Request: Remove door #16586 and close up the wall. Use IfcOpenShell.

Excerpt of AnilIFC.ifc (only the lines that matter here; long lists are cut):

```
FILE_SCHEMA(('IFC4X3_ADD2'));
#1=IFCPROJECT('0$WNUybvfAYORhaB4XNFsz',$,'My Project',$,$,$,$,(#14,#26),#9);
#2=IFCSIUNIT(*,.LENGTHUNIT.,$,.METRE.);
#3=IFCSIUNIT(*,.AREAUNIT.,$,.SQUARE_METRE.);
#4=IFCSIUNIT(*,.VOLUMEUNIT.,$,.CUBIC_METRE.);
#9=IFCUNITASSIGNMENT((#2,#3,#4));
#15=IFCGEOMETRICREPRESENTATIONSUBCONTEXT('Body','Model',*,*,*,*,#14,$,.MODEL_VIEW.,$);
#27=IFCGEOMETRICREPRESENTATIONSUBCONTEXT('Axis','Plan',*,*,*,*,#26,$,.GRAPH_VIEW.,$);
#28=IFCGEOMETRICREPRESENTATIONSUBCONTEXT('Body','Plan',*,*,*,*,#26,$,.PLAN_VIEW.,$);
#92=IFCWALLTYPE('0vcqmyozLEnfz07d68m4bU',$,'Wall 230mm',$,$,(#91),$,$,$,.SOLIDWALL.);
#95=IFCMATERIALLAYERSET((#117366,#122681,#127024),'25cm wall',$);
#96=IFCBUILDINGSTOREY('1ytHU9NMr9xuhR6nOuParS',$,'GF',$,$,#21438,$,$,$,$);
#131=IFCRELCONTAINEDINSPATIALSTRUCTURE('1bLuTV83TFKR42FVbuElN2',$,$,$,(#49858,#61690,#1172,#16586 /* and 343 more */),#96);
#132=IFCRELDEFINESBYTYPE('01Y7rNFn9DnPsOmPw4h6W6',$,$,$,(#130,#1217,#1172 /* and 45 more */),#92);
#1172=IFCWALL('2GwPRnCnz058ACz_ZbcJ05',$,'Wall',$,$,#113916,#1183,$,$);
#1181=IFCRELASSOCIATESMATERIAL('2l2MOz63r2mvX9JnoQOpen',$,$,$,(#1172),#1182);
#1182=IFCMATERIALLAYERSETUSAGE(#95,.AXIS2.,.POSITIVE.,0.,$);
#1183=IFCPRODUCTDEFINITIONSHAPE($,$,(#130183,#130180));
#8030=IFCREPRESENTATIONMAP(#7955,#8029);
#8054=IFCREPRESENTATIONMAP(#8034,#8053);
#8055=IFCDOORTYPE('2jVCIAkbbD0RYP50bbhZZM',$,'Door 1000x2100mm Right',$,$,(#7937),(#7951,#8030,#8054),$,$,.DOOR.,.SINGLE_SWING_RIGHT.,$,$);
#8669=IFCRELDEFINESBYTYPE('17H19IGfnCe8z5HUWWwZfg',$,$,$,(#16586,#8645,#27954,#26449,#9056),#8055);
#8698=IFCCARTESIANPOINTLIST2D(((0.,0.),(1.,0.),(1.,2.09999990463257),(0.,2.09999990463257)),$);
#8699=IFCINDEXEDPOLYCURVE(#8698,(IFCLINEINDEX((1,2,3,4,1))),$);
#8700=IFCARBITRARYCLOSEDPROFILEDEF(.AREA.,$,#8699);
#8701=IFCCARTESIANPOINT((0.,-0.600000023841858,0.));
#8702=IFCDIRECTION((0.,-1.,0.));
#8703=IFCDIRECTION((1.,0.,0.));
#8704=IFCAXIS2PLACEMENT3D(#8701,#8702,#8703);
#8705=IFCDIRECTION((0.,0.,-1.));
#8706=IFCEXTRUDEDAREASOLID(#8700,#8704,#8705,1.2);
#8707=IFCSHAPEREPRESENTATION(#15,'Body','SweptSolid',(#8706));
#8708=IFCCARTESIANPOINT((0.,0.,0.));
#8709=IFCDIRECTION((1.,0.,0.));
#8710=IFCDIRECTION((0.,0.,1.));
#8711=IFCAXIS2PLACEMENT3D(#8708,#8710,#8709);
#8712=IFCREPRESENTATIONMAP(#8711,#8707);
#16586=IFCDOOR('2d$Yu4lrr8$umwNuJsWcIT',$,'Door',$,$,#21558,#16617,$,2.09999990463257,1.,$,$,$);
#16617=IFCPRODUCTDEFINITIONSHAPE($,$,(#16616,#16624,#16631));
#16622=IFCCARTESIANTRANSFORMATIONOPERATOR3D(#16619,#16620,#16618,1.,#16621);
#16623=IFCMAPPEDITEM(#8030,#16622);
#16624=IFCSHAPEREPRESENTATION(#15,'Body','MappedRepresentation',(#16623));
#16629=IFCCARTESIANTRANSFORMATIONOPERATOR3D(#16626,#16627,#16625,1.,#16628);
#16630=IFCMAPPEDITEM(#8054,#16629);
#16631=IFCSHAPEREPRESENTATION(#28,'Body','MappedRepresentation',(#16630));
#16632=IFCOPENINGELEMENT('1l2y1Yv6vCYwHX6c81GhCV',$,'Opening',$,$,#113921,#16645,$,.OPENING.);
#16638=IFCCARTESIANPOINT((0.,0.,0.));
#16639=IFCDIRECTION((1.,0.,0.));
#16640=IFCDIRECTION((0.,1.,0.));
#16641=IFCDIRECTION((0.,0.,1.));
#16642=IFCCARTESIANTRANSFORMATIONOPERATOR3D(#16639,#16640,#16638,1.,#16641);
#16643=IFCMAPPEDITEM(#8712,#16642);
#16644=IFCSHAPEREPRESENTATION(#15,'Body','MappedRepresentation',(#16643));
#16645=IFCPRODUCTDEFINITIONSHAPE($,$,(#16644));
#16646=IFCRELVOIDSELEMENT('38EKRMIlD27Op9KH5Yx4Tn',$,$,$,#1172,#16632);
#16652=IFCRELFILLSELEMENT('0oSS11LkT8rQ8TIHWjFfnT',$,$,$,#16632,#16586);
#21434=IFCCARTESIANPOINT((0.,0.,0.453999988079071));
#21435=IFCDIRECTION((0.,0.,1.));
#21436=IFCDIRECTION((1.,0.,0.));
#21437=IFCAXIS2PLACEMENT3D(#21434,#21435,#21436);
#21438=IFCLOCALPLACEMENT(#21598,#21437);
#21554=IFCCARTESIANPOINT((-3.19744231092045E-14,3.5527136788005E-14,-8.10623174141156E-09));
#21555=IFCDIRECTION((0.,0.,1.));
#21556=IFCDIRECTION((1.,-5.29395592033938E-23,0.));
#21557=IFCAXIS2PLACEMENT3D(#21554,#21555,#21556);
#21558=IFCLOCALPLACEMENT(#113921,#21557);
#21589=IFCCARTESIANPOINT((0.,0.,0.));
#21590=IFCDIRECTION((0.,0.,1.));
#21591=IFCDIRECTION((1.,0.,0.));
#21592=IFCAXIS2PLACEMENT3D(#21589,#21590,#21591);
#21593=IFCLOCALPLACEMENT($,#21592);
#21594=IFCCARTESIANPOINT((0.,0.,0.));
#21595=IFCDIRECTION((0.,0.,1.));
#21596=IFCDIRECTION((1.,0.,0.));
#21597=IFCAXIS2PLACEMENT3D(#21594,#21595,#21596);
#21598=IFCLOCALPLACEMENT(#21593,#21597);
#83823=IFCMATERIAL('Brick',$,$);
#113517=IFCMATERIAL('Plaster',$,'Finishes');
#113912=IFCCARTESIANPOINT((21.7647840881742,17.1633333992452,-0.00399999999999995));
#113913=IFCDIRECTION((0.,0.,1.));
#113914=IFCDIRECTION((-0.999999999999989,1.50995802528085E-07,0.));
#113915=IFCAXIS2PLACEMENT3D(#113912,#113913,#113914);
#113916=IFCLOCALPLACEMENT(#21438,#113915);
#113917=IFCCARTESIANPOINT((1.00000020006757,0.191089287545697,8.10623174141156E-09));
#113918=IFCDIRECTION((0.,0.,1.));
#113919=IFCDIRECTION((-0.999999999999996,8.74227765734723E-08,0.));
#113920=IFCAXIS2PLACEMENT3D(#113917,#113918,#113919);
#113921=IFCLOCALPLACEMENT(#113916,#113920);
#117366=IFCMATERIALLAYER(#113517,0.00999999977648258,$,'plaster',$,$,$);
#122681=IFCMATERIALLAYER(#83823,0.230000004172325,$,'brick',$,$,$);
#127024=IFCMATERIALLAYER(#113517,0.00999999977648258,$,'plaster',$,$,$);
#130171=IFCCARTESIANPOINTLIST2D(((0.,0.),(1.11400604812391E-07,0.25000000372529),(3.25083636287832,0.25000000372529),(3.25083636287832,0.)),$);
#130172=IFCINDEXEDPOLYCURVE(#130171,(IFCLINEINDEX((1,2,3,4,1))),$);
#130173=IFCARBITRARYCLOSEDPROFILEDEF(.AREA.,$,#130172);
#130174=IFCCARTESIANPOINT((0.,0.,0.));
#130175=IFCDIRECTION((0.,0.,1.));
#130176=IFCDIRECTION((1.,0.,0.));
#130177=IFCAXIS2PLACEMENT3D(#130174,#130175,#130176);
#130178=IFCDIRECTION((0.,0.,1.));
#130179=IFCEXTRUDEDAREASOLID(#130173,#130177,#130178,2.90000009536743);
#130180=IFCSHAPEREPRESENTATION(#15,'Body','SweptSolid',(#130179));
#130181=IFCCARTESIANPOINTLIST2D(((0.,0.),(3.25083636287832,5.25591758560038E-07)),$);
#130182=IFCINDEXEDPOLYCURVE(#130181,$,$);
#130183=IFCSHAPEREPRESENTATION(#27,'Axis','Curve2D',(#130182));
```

```python
import ifcopenshell
import ifcopenshell.api.feature
import ifcopenshell.api.root
import ifcopenshell.geom
import ifcopenshell.util.shape

model = ifcopenshell.open("AnilIFC.ifc")
settings = ifcopenshell.geom.settings()


def volume(element):
    """Net volume in cubic metres, openings subtracted."""
    shape = ifcopenshell.geom.create_shape(settings, element)
    return ifcopenshell.util.shape.get_volume(shape.geometry)


door = model.by_guid("2d$Yu4lrr8$umwNuJsWcIT")
opening = door.FillsVoids[0].RelatingOpeningElement
wall = opening.VoidsElements[0].RelatingBuildingElement
before = volume(wall)

ifcopenshell.api.root.remove_product(model, product=door)
ifcopenshell.api.feature.remove_feature(model, feature=opening)

after = volume(wall)

print(f"wall volume {before:.3f} -> {after:.3f} m3")

model.write("AnilIFC_v2.ifc")
```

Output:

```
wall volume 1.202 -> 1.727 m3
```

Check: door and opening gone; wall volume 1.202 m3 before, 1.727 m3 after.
